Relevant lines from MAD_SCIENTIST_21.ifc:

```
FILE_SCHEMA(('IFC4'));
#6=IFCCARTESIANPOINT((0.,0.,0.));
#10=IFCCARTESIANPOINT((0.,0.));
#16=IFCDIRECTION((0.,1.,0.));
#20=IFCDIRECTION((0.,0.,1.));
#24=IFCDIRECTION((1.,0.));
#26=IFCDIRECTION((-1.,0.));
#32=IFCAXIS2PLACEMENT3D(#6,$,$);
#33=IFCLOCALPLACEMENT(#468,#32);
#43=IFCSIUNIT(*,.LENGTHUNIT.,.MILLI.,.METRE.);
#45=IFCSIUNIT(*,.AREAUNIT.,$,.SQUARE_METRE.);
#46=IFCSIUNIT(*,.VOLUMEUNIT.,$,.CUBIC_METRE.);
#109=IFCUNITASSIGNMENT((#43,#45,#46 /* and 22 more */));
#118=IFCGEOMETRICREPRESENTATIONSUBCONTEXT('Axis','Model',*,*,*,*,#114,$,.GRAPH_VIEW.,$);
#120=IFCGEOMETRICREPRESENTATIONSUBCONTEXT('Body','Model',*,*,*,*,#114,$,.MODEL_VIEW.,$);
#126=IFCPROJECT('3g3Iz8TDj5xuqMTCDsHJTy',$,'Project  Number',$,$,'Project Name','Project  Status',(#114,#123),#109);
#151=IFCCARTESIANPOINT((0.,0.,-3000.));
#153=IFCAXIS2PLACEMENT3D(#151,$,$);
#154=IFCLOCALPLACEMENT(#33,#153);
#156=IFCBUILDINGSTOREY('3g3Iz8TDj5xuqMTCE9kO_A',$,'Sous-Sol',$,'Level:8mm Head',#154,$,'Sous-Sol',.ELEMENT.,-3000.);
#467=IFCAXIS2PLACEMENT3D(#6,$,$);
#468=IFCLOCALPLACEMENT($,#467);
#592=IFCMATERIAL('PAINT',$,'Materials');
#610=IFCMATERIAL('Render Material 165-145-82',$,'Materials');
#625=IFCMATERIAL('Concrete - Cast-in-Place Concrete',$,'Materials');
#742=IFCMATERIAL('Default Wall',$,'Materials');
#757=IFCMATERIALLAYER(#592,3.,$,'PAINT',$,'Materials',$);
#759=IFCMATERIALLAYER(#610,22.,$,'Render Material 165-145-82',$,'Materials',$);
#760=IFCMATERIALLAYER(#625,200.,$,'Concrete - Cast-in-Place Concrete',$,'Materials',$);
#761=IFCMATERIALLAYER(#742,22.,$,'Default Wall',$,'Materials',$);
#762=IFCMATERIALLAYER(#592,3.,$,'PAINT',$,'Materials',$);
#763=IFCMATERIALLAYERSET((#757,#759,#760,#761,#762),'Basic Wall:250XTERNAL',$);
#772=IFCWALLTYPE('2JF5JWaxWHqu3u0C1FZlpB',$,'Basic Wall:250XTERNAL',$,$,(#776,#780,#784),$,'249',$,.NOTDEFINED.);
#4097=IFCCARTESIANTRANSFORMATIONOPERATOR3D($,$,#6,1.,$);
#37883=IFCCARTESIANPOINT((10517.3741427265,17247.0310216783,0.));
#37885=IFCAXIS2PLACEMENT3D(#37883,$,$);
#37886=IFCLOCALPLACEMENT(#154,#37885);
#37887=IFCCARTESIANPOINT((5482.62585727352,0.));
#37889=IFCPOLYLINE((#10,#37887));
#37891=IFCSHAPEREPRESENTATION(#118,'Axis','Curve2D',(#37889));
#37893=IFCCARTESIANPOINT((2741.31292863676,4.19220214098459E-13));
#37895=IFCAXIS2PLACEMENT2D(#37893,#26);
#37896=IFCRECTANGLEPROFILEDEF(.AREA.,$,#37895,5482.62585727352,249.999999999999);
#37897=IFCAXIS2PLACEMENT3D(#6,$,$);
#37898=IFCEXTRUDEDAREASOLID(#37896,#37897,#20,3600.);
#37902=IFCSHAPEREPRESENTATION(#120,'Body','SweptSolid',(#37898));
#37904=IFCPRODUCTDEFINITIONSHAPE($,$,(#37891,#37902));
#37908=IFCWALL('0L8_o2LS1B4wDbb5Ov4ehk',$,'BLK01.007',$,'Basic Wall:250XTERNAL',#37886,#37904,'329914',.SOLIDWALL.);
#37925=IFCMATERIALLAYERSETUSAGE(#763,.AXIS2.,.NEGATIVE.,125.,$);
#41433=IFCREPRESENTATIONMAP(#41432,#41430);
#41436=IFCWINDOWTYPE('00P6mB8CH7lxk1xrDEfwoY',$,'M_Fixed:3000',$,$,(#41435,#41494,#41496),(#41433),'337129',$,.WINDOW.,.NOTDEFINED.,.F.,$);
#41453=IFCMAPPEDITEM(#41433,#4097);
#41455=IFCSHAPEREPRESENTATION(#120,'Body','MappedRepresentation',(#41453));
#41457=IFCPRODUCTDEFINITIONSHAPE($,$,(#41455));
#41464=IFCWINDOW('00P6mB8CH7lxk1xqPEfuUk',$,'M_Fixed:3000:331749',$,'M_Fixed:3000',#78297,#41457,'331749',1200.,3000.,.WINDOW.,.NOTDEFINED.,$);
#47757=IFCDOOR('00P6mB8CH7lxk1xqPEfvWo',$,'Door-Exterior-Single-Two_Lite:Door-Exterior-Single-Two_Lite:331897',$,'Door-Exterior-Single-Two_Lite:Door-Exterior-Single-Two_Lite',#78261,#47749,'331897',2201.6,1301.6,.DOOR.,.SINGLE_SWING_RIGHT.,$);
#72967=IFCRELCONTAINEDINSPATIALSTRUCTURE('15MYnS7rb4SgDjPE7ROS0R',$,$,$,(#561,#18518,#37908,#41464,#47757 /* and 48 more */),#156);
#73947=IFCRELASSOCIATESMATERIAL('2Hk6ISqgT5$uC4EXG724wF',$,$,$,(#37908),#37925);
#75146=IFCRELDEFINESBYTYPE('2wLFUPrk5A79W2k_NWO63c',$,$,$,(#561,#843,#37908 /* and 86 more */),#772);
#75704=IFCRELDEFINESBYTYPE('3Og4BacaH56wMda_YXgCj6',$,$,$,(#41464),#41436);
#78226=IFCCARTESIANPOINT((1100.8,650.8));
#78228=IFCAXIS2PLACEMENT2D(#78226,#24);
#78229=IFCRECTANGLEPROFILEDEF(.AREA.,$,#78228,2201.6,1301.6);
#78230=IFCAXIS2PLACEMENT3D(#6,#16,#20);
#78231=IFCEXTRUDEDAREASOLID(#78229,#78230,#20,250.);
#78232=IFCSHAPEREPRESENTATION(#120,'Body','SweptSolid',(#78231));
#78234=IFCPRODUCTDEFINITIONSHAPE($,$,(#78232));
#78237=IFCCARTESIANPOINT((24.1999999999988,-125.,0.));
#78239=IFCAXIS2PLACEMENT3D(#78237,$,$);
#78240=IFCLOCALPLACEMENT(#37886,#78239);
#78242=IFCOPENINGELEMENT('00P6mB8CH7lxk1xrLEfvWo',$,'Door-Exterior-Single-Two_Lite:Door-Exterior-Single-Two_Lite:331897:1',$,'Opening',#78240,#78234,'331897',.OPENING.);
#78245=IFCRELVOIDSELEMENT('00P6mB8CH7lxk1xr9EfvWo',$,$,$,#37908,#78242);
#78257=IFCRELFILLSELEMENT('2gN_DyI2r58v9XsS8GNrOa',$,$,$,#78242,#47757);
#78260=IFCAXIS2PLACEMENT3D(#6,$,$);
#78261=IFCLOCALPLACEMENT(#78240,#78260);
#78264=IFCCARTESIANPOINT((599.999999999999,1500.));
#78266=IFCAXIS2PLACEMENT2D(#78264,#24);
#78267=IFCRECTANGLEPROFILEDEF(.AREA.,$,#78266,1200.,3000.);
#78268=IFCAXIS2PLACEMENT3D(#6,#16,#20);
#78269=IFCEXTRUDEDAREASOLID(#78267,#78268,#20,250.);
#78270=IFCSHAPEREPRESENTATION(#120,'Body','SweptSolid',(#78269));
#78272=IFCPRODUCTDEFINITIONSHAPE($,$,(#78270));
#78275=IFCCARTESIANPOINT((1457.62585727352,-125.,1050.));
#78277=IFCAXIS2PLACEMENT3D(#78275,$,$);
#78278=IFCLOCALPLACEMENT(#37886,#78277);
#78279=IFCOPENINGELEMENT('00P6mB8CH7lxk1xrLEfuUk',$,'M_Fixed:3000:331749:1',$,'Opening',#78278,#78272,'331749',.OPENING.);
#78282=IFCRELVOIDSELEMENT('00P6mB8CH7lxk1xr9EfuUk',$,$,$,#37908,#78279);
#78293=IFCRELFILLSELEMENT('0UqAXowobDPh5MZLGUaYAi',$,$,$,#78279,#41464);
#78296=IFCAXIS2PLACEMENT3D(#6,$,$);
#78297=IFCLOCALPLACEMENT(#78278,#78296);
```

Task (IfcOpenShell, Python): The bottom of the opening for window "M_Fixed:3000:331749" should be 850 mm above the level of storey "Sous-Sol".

```python
import numpy as np
import ifcopenshell
import ifcopenshell.api.geometry
import ifcopenshell.geom
import ifcopenshell.util.element
import ifcopenshell.util.placement
import ifcopenshell.util.shape
import ifcopenshell.util.unit

model = ifcopenshell.open("MAD_SCIENTIST_21.ifc")
unit_scale = ifcopenshell.util.unit.calculate_unit_scale(model)

window = model.by_guid("00P6mB8CH7lxk1xqPEfuUk")
opening = window.FillsVoids[0].RelatingOpeningElement
storey = ifcopenshell.util.element.get_container(window, ifc_class="IfcBuildingStorey")
level = ifcopenshell.util.placement.get_local_placement(storey.ObjectPlacement)[2, 3]

# The opening's origin need not be at the sill, so measure its lowest point.
shape = ifcopenshell.geom.create_shape(ifcopenshell.geom.settings(), opening)
bottom = ifcopenshell.util.shape.get_shape_bottom_elevation(shape, shape.geometry) / unit_scale
dz = level + 850.0 - bottom

shift = np.array([0.0, 0.0, dz])
# The window is placed relative to its opening, so it follows when the opening moves.
matrix = ifcopenshell.util.placement.get_local_placement(opening.ObjectPlacement)
matrix[:3, 3] += shift
ifcopenshell.api.geometry.edit_object_placement(
    model, product=opening, matrix=matrix, is_si=False, should_transform_children=True
)

print(f"moved by {dz * unit_scale:+.3f} m")

model.write("MAD_SCIENTIST_21_rev.ifc")
```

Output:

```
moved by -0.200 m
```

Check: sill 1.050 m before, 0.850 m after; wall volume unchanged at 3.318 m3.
